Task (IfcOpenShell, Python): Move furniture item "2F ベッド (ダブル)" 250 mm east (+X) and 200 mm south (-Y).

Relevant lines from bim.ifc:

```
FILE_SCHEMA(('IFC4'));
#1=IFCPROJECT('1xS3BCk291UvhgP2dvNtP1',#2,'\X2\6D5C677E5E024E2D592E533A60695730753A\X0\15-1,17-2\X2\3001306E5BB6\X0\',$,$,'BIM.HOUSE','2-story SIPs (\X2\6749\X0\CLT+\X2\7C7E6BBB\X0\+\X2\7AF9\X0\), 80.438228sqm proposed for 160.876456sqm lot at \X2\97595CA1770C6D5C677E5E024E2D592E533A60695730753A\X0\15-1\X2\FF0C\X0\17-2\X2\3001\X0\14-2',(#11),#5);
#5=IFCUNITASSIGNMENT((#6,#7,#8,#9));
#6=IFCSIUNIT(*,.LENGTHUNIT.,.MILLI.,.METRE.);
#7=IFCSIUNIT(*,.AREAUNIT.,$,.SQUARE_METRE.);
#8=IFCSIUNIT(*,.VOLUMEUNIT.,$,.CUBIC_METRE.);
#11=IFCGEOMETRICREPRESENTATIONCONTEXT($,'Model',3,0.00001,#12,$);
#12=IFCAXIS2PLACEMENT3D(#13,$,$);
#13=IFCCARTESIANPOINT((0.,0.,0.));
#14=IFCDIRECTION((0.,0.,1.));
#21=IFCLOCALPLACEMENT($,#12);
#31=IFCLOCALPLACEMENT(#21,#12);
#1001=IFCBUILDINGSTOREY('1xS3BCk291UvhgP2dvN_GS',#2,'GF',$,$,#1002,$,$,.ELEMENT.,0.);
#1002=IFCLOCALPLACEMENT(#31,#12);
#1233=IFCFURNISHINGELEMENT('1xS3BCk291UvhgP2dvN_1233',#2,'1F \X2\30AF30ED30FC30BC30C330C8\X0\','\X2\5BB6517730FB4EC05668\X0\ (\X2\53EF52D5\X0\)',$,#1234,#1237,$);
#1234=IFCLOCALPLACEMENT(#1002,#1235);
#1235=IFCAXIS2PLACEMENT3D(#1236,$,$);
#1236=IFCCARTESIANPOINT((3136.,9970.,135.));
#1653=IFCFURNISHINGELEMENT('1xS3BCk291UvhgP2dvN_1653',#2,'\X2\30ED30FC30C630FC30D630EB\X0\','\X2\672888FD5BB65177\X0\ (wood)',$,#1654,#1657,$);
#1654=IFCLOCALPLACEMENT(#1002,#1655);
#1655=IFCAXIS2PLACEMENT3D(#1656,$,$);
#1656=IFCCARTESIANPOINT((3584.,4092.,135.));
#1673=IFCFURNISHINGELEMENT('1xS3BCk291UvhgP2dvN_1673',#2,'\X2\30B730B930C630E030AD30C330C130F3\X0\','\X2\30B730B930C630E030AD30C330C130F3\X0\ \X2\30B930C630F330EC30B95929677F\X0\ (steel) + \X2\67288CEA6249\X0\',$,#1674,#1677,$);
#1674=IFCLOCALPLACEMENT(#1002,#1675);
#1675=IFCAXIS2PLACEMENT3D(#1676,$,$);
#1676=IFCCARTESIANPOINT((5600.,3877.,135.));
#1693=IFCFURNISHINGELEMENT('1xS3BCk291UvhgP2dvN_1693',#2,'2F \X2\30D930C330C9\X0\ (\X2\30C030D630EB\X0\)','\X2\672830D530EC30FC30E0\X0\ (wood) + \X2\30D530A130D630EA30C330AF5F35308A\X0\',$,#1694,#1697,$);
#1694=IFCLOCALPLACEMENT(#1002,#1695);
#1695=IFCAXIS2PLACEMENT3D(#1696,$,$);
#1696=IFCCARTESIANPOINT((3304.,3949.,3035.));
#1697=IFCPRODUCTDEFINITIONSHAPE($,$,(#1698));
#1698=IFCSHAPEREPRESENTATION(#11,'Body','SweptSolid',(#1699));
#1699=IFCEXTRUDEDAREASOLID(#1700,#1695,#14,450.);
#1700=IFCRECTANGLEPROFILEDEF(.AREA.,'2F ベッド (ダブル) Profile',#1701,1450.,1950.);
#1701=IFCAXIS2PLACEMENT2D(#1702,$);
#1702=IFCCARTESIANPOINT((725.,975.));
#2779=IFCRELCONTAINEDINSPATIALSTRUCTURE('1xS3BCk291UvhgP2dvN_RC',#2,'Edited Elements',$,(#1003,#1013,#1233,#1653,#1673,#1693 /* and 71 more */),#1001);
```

```python
import ifcopenshell
import ifcopenshell.api.geometry
import ifcopenshell.util.placement

model = ifcopenshell.open("bim.ifc")

item = model.by_guid("1xS3BCk291UvhgP2dvN_1693")
matrix = ifcopenshell.util.placement.get_local_placement(item.ObjectPlacement)
matrix[0, 3] += 250.0
matrix[1, 3] -= 200.0
ifcopenshell.api.geometry.edit_object_placement(model, product=item, matrix=matrix, is_si=False)

print(ifcopenshell.util.placement.get_local_placement(item.ObjectPlacement).round(3) + 0.0)

model.write("bim_v2.ifc")
```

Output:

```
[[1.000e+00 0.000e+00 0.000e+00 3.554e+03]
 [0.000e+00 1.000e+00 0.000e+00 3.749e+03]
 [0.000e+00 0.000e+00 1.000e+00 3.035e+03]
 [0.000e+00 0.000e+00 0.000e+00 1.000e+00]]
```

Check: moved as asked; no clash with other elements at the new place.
